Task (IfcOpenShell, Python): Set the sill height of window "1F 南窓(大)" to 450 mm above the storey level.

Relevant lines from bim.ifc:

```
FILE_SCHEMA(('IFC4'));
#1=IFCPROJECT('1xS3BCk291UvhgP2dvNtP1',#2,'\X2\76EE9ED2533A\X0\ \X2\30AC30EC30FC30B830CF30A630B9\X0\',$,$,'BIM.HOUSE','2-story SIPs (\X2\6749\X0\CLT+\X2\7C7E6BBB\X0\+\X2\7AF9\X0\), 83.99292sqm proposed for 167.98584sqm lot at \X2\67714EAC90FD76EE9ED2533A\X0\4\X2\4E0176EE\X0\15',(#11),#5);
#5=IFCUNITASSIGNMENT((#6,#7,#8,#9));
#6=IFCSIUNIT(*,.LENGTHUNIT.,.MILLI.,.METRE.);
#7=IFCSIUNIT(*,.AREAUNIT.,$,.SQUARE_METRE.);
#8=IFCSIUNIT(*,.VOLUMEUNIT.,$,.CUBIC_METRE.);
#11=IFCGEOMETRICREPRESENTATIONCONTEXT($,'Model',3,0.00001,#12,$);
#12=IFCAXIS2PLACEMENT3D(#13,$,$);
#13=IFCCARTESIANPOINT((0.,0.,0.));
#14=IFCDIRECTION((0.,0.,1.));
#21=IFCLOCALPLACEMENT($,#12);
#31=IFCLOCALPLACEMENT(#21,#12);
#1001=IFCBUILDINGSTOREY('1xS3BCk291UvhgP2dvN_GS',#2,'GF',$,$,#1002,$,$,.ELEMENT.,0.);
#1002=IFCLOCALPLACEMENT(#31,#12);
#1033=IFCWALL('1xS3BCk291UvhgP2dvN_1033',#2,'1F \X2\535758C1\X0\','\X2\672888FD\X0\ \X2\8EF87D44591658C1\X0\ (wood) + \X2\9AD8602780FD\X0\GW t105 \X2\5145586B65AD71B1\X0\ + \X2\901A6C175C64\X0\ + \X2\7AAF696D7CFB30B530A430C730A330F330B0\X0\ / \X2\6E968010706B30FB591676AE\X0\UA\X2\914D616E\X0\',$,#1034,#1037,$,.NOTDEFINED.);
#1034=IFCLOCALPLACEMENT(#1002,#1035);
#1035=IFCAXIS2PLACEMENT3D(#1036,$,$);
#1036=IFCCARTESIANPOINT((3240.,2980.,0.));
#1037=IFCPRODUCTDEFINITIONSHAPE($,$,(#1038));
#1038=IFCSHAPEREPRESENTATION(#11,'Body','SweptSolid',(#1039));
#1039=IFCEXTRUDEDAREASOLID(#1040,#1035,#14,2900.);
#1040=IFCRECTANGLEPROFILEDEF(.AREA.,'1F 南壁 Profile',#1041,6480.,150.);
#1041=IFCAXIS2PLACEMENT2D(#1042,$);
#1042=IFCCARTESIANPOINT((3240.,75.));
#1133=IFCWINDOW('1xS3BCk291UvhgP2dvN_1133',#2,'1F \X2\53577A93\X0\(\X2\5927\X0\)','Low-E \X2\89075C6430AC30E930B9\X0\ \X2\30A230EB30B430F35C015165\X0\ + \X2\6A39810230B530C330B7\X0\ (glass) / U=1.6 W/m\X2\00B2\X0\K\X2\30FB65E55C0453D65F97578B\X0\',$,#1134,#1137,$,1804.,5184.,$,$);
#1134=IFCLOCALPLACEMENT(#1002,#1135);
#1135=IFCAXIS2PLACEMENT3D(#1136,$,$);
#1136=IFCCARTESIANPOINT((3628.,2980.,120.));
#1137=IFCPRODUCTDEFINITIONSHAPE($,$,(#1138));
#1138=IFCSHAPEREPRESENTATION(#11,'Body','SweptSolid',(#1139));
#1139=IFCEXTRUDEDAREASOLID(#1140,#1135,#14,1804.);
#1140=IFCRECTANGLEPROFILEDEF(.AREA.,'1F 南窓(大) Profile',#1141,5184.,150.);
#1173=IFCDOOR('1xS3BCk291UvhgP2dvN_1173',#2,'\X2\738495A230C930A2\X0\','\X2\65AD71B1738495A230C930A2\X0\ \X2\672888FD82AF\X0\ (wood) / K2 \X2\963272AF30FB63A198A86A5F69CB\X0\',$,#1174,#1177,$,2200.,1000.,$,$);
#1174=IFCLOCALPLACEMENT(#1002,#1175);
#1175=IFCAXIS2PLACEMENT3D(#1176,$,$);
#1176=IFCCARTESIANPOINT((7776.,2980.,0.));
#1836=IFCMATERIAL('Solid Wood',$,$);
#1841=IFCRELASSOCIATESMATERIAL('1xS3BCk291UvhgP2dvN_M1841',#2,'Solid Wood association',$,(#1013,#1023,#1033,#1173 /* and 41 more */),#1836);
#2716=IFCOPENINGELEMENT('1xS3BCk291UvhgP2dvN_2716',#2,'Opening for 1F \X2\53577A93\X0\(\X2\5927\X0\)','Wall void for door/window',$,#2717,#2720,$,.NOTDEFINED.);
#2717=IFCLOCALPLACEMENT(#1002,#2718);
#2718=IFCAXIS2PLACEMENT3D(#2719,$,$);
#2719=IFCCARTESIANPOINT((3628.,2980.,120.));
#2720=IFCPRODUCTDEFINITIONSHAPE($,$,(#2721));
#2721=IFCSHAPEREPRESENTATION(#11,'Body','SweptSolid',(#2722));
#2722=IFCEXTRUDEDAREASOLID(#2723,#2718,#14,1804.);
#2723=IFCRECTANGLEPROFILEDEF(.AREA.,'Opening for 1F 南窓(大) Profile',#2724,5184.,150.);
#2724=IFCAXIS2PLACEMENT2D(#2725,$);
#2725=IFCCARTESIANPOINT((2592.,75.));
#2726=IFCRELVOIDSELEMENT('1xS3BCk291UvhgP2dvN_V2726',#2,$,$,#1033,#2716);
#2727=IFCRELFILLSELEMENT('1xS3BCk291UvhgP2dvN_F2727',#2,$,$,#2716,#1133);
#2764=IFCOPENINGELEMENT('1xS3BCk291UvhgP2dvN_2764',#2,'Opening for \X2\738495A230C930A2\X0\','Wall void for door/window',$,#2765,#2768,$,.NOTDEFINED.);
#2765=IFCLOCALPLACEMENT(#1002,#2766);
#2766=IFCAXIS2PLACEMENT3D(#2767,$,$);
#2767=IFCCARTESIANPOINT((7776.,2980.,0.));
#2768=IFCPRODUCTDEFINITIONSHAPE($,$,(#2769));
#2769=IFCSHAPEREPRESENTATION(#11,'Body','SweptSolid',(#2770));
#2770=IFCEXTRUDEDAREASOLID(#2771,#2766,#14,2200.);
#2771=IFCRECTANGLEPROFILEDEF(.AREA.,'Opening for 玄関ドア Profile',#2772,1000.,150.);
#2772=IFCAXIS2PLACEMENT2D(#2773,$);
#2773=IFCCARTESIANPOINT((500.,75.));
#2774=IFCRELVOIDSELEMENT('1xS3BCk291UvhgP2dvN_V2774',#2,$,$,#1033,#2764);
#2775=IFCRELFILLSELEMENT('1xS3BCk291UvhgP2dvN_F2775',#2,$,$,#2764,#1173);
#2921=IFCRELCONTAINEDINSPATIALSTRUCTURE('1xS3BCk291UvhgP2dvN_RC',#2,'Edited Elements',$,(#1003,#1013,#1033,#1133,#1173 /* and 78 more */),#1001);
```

```python
import numpy as np
import ifcopenshell
import ifcopenshell.api.geometry
import ifcopenshell.geom
import ifcopenshell.util.element
import ifcopenshell.util.placement
import ifcopenshell.util.shape
import ifcopenshell.util.unit

model = ifcopenshell.open("bim.ifc")
unit_scale = ifcopenshell.util.unit.calculate_unit_scale(model)

window = model.by_guid("1xS3BCk291UvhgP2dvN_1133")
opening = window.FillsVoids[0].RelatingOpeningElement
storey = ifcopenshell.util.element.get_container(window, ifc_class="IfcBuildingStorey")
level = ifcopenshell.util.placement.get_local_placement(storey.ObjectPlacement)[2, 3]

# The opening's origin need not be at the sill, so measure its lowest point.
shape = ifcopenshell.geom.create_shape(ifcopenshell.geom.settings(), opening)
bottom = ifcopenshell.util.shape.get_shape_bottom_elevation(shape, shape.geometry) / unit_scale
dz = level + 450.0 - bottom

shift = np.array([0.0, 0.0, dz])
# The window is not placed relative to its opening, so move both.
for product in (opening, window):
    matrix = ifcopenshell.util.placement.get_local_placement(product.ObjectPlacement)
    matrix[:3, 3] += shift
    ifcopenshell.api.geometry.edit_object_placement(model, product=product, matrix=matrix, is_si=False)

print(f"moved by {dz * unit_scale:+.3f} m")

model.write("bim-out.ifc")
```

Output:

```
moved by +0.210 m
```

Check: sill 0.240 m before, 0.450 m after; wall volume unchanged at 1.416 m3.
